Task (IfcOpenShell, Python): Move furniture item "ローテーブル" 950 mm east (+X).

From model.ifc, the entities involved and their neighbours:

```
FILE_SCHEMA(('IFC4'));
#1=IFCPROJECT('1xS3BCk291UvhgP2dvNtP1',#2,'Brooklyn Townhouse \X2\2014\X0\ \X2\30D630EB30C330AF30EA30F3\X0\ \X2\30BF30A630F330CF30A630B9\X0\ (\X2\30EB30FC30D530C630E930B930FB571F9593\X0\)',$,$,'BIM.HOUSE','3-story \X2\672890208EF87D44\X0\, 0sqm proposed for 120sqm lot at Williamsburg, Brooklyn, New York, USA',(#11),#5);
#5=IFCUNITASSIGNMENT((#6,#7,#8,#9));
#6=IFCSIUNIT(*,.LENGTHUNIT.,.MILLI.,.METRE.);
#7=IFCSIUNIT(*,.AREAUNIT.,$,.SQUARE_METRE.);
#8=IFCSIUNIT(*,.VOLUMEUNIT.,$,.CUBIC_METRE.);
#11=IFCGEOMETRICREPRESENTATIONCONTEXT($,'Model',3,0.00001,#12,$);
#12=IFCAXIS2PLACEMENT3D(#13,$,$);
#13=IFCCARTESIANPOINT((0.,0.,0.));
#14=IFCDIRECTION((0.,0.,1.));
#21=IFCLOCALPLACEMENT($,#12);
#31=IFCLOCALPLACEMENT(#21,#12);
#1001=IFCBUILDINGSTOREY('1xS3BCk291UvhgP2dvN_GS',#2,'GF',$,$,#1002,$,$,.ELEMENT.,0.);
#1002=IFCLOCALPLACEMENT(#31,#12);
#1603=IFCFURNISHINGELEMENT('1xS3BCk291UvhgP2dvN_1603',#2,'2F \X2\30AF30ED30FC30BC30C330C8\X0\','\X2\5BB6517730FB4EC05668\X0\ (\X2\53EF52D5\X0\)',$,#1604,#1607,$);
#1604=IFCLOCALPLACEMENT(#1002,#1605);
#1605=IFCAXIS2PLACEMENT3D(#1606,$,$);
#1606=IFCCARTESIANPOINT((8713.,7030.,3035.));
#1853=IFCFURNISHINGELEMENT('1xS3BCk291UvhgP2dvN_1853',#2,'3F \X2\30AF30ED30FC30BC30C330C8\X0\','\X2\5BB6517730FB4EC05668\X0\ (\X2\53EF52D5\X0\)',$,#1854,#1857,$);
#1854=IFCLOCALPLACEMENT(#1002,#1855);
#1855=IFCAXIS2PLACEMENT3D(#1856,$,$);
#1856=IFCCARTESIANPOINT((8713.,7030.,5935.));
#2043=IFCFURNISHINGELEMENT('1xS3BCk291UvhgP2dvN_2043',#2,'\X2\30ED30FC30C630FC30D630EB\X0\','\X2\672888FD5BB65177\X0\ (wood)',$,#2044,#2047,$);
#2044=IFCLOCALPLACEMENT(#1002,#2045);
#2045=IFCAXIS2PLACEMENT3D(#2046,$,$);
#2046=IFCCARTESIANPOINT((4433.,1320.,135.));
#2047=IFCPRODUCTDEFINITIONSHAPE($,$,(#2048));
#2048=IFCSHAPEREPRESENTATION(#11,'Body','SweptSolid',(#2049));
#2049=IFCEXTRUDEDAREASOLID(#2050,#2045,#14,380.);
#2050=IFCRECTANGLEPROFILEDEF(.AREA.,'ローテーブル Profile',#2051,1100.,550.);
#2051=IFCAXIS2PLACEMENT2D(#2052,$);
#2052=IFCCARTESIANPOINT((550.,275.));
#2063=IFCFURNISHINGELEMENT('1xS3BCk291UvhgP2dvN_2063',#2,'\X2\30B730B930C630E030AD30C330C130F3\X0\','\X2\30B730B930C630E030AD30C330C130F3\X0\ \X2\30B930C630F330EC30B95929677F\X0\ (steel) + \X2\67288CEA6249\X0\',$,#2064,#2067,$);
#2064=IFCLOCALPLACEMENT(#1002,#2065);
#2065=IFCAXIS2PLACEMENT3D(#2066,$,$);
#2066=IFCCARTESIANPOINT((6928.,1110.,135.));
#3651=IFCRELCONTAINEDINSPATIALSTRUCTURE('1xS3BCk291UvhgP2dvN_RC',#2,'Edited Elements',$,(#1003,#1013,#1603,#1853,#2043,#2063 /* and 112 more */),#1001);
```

```python
import ifcopenshell
import ifcopenshell.api.geometry
import ifcopenshell.util.placement
import ifcopenshell.util.unit

model = ifcopenshell.open("model.ifc")
unit_scale = ifcopenshell.util.unit.calculate_unit_scale(model)

item = model.by_guid("1xS3BCk291UvhgP2dvN_2043")
matrix = ifcopenshell.util.placement.get_local_placement(item.ObjectPlacement)
matrix[0, 3] += 0.95 / unit_scale
ifcopenshell.api.geometry.edit_object_placement(model, product=item, matrix=matrix, is_si=False)

print(ifcopenshell.util.placement.get_local_placement(item.ObjectPlacement).round(3) + 0.0)

model.write("model_v2.ifc")
```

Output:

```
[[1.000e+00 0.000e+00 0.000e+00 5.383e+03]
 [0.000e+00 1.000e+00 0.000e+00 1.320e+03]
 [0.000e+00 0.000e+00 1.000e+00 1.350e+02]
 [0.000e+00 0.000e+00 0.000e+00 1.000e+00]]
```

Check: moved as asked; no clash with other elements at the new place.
